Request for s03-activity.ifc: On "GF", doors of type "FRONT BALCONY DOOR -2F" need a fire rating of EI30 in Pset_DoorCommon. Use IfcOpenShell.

First a look at what the model holds.

```python
import ifcopenshell
import ifcopenshell.util.element

model = ifcopenshell.open("s03-activity.ifc")
print(model.schema)
storey = next(s for s in model.by_type("IfcBuildingStorey") if s.Name == "GF")
doors = [e for e in ifcopenshell.util.element.get_decomposition(storey) if e.is_a("IfcDoor")]
seen = {}
for e in doors:
    element_type = ifcopenshell.util.element.get_type(e)
    key = (element_type.Name if element_type != e and element_type else None, ifcopenshell.util.element.get_pset(e, "Pset_DoorCommon", "FireRating"))
    seen[key] = seen.get(key, 0) + 1
for (name, value), count in sorted(seen.items(), key=str):
    print(count, "x", name, "|", value)
```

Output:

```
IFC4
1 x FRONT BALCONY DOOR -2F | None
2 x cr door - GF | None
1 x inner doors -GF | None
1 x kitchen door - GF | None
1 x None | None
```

```python
import ifcopenshell
import ifcopenshell.api.pset
import ifcopenshell.util.element

model = ifcopenshell.open("s03-activity.ifc")

storey = next(s for s in model.by_type("IfcBuildingStorey") if s.Name == "GF")
doors = [e for e in ifcopenshell.util.element.get_decomposition(storey) if e.is_a("IfcDoor")]

count = 0
for e in doors:
    element_type = ifcopenshell.util.element.get_type(e)
    if element_type in (None, e) or element_type.Name != "FRONT BALCONY DOOR -2F":
        continue
    # add_pset returns the element's existing set when there is one.
    pset = ifcopenshell.api.pset.add_pset(model, product=e, name="Pset_DoorCommon")
    ifcopenshell.api.pset.edit_pset(model, pset=pset, properties={"FireRating": "EI30"})
    count += 1

print(count, "doors updated")

model.write("s03-activity-out.ifc")
```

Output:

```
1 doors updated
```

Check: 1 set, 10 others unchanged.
